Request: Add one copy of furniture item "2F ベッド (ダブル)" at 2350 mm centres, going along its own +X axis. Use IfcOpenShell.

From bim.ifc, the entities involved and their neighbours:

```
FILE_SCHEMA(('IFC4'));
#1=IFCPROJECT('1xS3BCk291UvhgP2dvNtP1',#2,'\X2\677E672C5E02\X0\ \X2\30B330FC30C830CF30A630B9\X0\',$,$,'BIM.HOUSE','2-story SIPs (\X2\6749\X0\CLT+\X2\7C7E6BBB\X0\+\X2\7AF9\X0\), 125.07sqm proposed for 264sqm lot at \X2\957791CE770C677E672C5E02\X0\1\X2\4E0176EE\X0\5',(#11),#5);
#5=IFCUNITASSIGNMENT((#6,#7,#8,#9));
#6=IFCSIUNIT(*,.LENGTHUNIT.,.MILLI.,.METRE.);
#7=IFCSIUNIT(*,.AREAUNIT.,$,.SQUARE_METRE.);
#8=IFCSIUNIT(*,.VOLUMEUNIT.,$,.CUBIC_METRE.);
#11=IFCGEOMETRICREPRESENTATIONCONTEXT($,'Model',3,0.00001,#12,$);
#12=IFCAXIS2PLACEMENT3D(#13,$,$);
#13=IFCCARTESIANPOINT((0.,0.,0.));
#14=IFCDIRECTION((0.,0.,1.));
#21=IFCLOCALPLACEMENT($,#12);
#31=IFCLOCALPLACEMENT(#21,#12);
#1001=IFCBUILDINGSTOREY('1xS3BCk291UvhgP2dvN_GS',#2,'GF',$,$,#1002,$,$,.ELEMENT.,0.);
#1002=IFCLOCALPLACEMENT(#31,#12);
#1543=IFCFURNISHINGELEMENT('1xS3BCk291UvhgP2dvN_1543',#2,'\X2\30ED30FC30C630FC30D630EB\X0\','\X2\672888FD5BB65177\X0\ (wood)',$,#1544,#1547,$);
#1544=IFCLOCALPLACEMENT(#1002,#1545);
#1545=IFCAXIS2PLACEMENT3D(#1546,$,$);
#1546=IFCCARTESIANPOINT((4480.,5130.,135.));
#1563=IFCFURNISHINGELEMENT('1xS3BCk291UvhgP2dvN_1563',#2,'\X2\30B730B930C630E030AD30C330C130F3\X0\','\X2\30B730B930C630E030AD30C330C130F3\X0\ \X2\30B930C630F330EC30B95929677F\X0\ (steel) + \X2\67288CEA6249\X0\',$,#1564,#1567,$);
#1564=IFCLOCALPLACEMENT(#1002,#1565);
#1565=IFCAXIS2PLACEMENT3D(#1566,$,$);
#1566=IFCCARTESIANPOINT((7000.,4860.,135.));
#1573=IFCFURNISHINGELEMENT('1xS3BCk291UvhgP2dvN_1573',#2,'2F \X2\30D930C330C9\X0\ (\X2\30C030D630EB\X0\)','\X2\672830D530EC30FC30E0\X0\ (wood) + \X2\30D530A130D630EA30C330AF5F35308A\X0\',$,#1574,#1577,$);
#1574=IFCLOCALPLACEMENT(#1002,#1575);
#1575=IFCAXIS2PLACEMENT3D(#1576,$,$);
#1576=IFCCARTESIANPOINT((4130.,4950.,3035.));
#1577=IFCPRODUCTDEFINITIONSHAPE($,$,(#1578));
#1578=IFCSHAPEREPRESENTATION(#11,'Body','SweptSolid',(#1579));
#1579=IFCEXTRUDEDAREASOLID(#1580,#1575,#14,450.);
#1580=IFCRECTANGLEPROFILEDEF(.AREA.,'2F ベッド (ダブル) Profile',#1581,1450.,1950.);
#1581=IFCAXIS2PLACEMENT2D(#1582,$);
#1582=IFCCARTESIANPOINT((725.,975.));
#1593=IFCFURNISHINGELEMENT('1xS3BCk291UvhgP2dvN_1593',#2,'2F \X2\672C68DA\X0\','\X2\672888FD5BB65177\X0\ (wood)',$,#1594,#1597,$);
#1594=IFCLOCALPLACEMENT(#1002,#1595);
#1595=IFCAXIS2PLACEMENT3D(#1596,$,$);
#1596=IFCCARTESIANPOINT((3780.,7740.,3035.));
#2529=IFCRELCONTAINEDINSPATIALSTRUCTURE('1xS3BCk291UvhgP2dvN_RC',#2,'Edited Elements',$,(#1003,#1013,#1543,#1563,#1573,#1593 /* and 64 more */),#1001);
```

```python
import ifcopenshell
import ifcopenshell.api.geometry
import ifcopenshell.api.root
import ifcopenshell.util.element
import ifcopenshell.util.placement
import ifcopenshell.util.unit

model = ifcopenshell.open("bim.ifc")
unit_scale = ifcopenshell.util.unit.calculate_unit_scale(model)


def reuse_history(source, copy):
    """copy_class also copies each property set's owner history, people and application; keep the originals."""
    for rel in copy.IsDefinedBy:
        if rel.is_a("IfcRelDefinesByProperties") and (history := rel.RelatingPropertyDefinition.OwnerHistory):
            rel.RelatingPropertyDefinition.OwnerHistory = source.OwnerHistory
            ifcopenshell.util.element.remove_deep2(model, history)


source = model.by_guid("1xS3BCk291UvhgP2dvN_1573")
base = ifcopenshell.util.placement.get_local_placement(source.ObjectPlacement)
step = base[:3, 0] * 2.35 / unit_scale

for i in range(1, 2):
    copy = ifcopenshell.api.root.copy_class(model, product=source)
    copy.Representation = ifcopenshell.util.element.copy_deep(
        model, source.Representation, exclude=["IfcGeometricRepresentationContext", "IfcRepresentationMap"]
    )
    reuse_history(source, copy)
    matrix = base.copy()
    matrix[:3, 3] += i * step
    print("added at", matrix[:3, 3].round(3) + 0.0)
    ifcopenshell.api.geometry.edit_object_placement(model, product=copy, matrix=matrix, is_si=False)

model.write("bim_updated.ifc")
```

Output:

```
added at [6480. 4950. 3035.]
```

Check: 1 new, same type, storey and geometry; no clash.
